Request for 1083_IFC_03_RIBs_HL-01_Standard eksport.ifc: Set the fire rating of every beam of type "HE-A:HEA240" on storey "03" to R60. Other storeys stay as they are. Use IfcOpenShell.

First a look at what the model holds.

```python
import ifcopenshell
import ifcopenshell.util.element

model = ifcopenshell.open("1083_IFC_03_RIBs_HL-01_Standard eksport.ifc")
print(model.schema)
storey = next(s for s in model.by_type("IfcBuildingStorey") if s.Name == "03")
beams = [e for e in ifcopenshell.util.element.get_decomposition(storey) if e.is_a("IfcBeam")]
seen = {}
for e in beams:
    element_type = ifcopenshell.util.element.get_type(e)
    key = (element_type.Name if element_type != e and element_type else None, ifcopenshell.util.element.get_pset(e, "Pset_BeamCommon", "FireRating"))
    seen[key] = seen.get(key, 0) + 1
for (name, value), count in sorted(seen.items(), key=str):
    print(count, "x", name, "|", value)
```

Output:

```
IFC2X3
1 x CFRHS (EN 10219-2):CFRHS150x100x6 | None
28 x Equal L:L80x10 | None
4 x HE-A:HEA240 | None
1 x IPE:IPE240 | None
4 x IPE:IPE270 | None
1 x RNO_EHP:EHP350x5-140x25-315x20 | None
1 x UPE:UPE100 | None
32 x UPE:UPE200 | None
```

```python
import ifcopenshell
import ifcopenshell.api.pset
import ifcopenshell.util.element

model = ifcopenshell.open("1083_IFC_03_RIBs_HL-01_Standard eksport.ifc")

storey = next(s for s in model.by_type("IfcBuildingStorey") if s.Name == "03")
beams = [e for e in ifcopenshell.util.element.get_decomposition(storey) if e.is_a("IfcBeam")]

count = 0
for e in beams:
    element_type = ifcopenshell.util.element.get_type(e)
    if element_type in (None, e) or element_type.Name != "HE-A:HEA240":
        continue
    # add_pset returns the element's existing set when there is one.
    pset = ifcopenshell.api.pset.add_pset(model, product=e, name="Pset_BeamCommon")
    ifcopenshell.api.pset.edit_pset(model, pset=pset, properties={"FireRating": "R60"})
    count += 1

print(count, "beams updated")

model.write("1083_IFC_03_RIBs_HL-01_Standard eksport_updated.ifc")
```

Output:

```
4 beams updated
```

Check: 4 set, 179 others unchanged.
